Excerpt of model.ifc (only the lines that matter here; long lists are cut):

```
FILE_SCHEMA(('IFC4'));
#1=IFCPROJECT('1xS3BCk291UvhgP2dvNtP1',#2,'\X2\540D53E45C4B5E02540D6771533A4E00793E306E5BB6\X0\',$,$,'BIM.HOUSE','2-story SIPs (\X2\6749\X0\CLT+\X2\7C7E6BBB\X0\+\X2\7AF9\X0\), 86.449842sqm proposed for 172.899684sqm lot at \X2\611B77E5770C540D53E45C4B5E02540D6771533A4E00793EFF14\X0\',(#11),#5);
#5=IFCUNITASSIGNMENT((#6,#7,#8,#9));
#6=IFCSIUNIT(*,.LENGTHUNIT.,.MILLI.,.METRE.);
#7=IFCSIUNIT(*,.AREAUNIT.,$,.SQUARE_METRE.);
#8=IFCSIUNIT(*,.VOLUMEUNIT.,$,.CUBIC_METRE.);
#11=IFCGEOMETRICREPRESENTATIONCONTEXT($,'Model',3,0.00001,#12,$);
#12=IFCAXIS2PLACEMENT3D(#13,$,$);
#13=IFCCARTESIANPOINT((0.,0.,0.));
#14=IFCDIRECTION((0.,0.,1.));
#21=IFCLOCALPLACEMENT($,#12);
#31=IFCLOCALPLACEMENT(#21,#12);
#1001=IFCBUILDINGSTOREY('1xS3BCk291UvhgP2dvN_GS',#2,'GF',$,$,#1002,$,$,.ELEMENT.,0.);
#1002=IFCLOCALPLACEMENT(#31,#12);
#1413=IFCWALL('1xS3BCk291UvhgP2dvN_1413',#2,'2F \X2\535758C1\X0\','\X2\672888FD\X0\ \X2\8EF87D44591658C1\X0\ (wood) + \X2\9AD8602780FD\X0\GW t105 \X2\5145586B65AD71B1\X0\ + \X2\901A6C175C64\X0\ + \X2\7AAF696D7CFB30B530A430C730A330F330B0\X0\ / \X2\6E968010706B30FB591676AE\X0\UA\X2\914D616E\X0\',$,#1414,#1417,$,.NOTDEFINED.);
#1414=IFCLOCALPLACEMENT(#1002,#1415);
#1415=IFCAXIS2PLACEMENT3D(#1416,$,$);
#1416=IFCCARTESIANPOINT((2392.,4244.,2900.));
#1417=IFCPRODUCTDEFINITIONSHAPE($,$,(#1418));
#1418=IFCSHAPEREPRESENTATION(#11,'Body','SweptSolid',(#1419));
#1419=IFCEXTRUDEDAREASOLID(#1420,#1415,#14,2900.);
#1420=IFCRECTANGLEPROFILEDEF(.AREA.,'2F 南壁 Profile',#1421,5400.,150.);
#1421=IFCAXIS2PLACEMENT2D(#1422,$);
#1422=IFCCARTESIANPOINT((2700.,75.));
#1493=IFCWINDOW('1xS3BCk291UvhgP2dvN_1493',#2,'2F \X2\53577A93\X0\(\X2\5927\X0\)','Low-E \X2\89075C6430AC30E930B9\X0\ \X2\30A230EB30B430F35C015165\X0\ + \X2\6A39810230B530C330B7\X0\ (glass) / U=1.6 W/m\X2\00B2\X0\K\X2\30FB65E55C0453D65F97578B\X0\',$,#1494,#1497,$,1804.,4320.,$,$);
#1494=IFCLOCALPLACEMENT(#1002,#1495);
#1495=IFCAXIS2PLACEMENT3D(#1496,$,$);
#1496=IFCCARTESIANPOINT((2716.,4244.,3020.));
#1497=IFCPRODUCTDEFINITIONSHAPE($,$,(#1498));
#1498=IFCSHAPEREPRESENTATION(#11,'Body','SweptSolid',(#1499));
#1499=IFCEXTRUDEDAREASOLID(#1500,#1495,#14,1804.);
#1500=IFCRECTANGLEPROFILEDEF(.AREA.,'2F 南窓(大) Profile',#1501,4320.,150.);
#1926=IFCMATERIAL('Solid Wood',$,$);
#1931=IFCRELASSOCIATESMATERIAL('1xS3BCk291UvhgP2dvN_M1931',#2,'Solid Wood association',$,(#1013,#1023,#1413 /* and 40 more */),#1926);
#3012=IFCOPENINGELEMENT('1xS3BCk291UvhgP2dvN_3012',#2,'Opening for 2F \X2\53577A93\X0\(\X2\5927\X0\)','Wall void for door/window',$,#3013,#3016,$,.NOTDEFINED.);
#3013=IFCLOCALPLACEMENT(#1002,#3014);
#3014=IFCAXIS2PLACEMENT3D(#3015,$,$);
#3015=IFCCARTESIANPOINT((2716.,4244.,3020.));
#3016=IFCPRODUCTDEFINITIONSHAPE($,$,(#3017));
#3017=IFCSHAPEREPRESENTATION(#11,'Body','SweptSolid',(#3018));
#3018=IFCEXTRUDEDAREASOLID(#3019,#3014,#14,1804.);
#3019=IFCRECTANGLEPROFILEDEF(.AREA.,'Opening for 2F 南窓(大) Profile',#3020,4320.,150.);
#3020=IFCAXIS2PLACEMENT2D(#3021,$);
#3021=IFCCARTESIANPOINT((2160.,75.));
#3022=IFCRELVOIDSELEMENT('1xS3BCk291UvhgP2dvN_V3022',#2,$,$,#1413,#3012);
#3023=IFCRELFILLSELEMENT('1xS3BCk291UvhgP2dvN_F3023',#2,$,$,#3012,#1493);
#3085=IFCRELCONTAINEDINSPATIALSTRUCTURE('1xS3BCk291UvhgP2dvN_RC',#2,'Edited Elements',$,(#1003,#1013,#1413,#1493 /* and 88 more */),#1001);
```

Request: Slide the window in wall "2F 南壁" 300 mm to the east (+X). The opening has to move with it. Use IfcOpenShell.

```python
import ifcopenshell
import ifcopenshell.api.geometry
import ifcopenshell.util.placement
import ifcopenshell.util.unit

model = ifcopenshell.open("model.ifc")
unit_scale = ifcopenshell.util.unit.calculate_unit_scale(model)

window = model.by_guid("1xS3BCk291UvhgP2dvN_1493")
opening = window.FillsVoids[0].RelatingOpeningElement
wall = opening.VoidsElements[0].RelatingBuildingElement

wall_matrix = ifcopenshell.util.placement.get_local_placement(wall.ObjectPlacement)
shift = wall_matrix[:3, 0] * 0.3 / unit_scale
before = ifcopenshell.util.placement.get_local_placement(window.ObjectPlacement)[:3, 3].copy()

# The window is not placed relative to its opening, so move both.
for product in (opening, window):
    matrix = ifcopenshell.util.placement.get_local_placement(product.ObjectPlacement)
    matrix[:3, 3] += shift
    ifcopenshell.api.geometry.edit_object_placement(model, product=product, matrix=matrix, is_si=False)

after = ifcopenshell.util.placement.get_local_placement(window.ObjectPlacement)[:3, 3]
print("window moved by", (after - before).round(3) + 0.0)

model.write("model_rev.ifc")
```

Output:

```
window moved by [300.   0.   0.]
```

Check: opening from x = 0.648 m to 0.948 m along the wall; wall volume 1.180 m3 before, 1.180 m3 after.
